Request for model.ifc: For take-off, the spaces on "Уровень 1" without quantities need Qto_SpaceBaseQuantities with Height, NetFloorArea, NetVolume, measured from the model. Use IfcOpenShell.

First a look at what the model holds.

```python
import ifcopenshell
import ifcopenshell.util.element
import ifcopenshell.util.unit

model = ifcopenshell.open("model.ifc")
print(model.schema)
for unit_type in ("LENGTHUNIT", "AREAUNIT", "VOLUMEUNIT"):
    print(unit_type, ifcopenshell.util.unit.calculate_unit_scale(model, unit_type))
storey = next(s for s in model.by_type("IfcBuildingStorey") if s.Name == "Уровень 1")
spaces = [e for e in ifcopenshell.util.element.get_decomposition(storey) if e.is_a("IfcSpace")]
for e in sorted(spaces, key=lambda e: e.id()):
    print(e.id(), e.is_a(), e.Name, list(ifcopenshell.util.element.get_psets(e, qtos_only=True)), sep=" | ")
```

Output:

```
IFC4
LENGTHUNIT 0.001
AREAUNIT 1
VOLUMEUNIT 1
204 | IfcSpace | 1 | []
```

```python
import ifcopenshell
import ifcopenshell.api.pset
import ifcopenshell.geom
import ifcopenshell.util.element
import ifcopenshell.util.shape
import ifcopenshell.util.unit

model = ifcopenshell.open("model.ifc")
unit_scale = ifcopenshell.util.unit.calculate_unit_scale(model)
area_scale = ifcopenshell.util.unit.calculate_unit_scale(model, "AREAUNIT")
volume_scale = ifcopenshell.util.unit.calculate_unit_scale(model, "VOLUMEUNIT")
settings = ifcopenshell.geom.settings()

storey = next(s for s in model.by_type("IfcBuildingStorey") if s.Name == "Уровень 1")
spaces = [e for e in ifcopenshell.util.element.get_decomposition(storey) if e.is_a("IfcSpace")]

for e in sorted(spaces, key=lambda e: e.id()):
    if ifcopenshell.util.element.get_psets(e, qtos_only=True, should_inherit=False):
        continue
    # Geometry comes back in metres, in the element's own axes.
    shape = ifcopenshell.geom.create_shape(settings, e)
    values = {
        "Height": ifcopenshell.util.shape.get_z(shape.geometry) / unit_scale,
        "NetFloorArea": ifcopenshell.util.shape.get_footprint_area(shape.geometry) / area_scale,
        "NetVolume": ifcopenshell.util.shape.get_volume(shape.geometry) / volume_scale,
    }
    qto = ifcopenshell.api.pset.add_qto(model, product=e, name="Qto_SpaceBaseQuantities")
    ifcopenshell.api.pset.edit_qto(model, qto=qto, properties=values)
    print(e.id(), {k: round(v, 3) for k, v in values.items()})

model.write("model-out.ifc")
```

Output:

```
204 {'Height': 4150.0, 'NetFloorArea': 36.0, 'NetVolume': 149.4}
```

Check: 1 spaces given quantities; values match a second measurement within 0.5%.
